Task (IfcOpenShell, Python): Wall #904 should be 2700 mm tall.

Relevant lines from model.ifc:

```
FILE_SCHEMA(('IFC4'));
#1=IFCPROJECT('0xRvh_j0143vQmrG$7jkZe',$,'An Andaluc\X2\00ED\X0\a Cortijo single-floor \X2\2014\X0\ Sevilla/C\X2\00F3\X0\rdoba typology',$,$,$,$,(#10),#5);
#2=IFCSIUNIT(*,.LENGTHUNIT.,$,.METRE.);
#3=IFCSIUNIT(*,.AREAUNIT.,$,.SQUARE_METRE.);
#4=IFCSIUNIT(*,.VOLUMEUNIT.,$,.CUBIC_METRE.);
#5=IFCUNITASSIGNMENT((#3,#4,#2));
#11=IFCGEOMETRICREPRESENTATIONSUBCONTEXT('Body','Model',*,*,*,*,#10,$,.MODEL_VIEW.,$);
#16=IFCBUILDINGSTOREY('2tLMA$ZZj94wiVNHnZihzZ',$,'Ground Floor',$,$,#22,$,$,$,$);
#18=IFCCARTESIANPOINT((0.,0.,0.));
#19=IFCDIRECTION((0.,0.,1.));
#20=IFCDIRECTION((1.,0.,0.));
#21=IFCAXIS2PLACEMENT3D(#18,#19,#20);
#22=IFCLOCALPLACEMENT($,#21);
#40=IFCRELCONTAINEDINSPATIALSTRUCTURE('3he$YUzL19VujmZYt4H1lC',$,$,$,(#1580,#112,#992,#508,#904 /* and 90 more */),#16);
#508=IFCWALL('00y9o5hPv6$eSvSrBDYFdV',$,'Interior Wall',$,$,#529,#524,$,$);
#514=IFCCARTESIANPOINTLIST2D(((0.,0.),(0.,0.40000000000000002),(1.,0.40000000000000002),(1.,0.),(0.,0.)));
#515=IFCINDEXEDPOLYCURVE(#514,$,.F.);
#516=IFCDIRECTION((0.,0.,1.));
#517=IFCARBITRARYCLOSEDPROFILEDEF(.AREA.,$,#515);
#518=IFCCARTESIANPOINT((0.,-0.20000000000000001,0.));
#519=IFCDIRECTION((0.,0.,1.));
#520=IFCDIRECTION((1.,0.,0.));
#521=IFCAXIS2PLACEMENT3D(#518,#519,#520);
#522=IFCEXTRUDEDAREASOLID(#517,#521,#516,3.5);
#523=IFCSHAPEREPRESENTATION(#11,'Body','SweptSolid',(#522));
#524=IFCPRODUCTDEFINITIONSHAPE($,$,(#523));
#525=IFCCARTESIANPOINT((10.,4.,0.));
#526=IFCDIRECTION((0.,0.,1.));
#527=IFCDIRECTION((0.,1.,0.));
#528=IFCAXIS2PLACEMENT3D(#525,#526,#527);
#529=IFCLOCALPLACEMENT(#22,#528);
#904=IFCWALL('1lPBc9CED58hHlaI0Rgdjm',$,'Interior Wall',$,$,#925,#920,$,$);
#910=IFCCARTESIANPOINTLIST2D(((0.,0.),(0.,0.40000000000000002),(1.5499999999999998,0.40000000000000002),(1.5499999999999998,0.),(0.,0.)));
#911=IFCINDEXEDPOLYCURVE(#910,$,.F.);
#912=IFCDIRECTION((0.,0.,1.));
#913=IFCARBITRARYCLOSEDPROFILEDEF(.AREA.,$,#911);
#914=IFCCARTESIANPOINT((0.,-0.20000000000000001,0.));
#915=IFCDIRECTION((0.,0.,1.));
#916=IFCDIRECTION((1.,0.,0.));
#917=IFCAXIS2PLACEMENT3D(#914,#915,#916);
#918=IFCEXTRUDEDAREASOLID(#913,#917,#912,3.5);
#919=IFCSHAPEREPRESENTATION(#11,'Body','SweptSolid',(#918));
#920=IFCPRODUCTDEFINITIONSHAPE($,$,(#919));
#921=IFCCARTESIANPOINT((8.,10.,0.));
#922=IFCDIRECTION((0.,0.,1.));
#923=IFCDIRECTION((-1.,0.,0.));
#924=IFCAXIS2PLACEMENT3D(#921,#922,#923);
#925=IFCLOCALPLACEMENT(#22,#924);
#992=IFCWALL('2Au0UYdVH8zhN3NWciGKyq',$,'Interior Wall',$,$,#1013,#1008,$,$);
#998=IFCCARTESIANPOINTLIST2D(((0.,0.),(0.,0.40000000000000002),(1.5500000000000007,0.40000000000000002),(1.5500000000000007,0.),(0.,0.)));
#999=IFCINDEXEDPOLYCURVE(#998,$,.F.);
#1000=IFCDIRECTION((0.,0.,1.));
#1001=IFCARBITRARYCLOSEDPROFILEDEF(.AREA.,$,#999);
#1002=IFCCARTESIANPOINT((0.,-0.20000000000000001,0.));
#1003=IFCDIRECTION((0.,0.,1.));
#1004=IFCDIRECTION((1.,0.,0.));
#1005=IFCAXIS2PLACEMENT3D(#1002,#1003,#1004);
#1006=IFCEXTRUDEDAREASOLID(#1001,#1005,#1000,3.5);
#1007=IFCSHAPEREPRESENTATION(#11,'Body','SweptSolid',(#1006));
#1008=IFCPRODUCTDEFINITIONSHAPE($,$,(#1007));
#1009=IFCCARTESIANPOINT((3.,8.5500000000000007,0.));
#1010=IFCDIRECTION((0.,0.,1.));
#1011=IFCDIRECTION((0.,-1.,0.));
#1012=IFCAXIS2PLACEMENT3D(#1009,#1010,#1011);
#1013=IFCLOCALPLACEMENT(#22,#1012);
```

```python
import ifcopenshell
import ifcopenshell.geom
import ifcopenshell.util.representation
import ifcopenshell.util.shape

model = ifcopenshell.open("model.ifc")
settings = ifcopenshell.geom.settings()


def volume(element):
    """Net volume in cubic metres, openings subtracted."""
    shape = ifcopenshell.geom.create_shape(settings, element)
    return ifcopenshell.util.shape.get_volume(shape.geometry)


wall = model.by_guid("1lPBc9CED58hHlaI0Rgdjm")
before = volume(wall)

body = ifcopenshell.util.representation.get_representation(wall, "Model", "Body")
solid = body.Items[0]
old_height = solid.Depth
solid.Depth = 2.7
after = volume(wall)

print(f"height {old_height:g} -> {solid.Depth:g}, volume {before:.3f} -> {after:.3f} m3")

model.write("model_rev.ifc")
```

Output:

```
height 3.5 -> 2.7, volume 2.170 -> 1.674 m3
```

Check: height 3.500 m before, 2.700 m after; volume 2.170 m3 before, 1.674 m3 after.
